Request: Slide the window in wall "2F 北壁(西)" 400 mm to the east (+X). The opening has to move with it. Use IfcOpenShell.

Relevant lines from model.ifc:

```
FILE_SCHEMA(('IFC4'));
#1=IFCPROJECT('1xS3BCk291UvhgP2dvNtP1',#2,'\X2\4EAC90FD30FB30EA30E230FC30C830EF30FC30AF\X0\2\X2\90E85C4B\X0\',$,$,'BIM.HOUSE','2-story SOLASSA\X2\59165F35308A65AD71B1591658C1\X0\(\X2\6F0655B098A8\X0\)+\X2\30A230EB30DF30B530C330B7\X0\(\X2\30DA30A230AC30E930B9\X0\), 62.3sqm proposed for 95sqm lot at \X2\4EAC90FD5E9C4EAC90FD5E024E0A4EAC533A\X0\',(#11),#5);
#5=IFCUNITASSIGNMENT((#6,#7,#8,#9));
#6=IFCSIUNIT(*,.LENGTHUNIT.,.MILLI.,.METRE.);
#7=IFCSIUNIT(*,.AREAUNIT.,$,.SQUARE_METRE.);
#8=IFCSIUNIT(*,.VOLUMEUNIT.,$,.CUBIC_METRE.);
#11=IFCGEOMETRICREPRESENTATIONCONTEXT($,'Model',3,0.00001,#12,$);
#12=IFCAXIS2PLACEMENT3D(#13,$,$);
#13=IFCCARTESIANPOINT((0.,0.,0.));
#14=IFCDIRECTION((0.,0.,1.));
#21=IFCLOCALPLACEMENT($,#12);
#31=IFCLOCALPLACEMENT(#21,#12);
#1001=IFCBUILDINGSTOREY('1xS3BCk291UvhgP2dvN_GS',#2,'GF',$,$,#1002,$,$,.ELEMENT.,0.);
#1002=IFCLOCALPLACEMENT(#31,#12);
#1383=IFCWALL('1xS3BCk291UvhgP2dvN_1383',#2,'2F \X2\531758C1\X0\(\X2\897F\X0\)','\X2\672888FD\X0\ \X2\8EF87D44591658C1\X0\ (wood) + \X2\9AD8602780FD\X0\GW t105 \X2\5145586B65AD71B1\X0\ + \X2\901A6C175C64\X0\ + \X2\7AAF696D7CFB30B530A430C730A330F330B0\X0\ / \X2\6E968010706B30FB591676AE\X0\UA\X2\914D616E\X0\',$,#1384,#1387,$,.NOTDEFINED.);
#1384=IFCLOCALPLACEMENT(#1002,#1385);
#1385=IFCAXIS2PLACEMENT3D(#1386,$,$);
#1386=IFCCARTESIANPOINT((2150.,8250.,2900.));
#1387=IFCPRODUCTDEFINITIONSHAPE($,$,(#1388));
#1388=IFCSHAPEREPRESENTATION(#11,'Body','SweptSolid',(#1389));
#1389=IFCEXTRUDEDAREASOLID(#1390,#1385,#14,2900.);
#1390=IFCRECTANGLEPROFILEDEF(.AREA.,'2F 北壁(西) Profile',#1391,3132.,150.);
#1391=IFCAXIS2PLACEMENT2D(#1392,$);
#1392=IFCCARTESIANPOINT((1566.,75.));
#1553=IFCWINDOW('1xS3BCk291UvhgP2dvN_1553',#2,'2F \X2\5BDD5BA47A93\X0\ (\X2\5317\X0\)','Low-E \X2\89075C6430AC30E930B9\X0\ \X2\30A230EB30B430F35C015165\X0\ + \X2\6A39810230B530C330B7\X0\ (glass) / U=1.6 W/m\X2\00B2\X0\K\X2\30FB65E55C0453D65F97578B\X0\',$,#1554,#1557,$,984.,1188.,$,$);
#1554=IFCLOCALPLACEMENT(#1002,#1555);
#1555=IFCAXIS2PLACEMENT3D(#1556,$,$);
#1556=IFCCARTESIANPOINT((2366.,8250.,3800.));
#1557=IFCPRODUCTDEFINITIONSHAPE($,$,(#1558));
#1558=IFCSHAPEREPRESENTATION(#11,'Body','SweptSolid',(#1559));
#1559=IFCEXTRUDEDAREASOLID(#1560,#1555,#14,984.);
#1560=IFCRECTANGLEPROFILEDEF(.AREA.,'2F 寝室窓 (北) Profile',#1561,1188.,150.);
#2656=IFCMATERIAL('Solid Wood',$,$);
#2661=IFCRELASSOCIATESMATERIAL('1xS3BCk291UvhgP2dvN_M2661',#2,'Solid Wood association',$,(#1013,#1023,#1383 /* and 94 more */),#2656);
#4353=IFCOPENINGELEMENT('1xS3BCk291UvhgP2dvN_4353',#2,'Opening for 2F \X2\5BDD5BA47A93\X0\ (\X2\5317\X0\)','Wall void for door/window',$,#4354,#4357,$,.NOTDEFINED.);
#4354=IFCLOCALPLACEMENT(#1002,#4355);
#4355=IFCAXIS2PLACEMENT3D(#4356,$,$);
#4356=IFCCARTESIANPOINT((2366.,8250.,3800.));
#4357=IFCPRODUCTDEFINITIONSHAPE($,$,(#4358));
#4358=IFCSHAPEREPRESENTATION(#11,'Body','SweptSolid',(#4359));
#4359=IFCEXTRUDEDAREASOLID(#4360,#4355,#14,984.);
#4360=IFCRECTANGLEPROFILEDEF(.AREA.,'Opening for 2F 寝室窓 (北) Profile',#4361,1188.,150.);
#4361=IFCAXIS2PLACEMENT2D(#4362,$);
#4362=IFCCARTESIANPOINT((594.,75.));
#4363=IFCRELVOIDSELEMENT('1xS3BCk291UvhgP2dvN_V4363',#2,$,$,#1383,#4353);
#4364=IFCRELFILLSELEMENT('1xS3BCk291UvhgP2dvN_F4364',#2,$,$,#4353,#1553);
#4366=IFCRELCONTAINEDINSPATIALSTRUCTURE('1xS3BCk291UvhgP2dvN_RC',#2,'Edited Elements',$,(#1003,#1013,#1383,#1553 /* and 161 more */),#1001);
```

```python
import ifcopenshell
import ifcopenshell.api.geometry
import ifcopenshell.util.placement
import ifcopenshell.util.unit

model = ifcopenshell.open("model.ifc")
unit_scale = ifcopenshell.util.unit.calculate_unit_scale(model)

window = model.by_guid("1xS3BCk291UvhgP2dvN_1553")
opening = window.FillsVoids[0].RelatingOpeningElement
wall = opening.VoidsElements[0].RelatingBuildingElement

wall_matrix = ifcopenshell.util.placement.get_local_placement(wall.ObjectPlacement)
shift = wall_matrix[:3, 0] * 0.4 / unit_scale
before = ifcopenshell.util.placement.get_local_placement(window.ObjectPlacement)[:3, 3].copy()

# The window is not placed relative to its opening, so move both.
for product in (opening, window):
    matrix = ifcopenshell.util.placement.get_local_placement(product.ObjectPlacement)
    matrix[:3, 3] += shift
    ifcopenshell.api.geometry.edit_object_placement(model, product=product, matrix=matrix, is_si=False)

after = ifcopenshell.util.placement.get_local_placement(window.ObjectPlacement)[:3, 3]
print("window moved by", (after - before).round(3) + 0.0)

model.write("model_rev.ifc")
```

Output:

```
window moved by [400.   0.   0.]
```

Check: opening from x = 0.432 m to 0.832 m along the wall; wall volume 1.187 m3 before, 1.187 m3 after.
